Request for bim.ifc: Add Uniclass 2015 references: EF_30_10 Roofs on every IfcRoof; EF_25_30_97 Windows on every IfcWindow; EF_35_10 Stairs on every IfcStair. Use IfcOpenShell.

First a look at what the model holds.

```python
import ifcopenshell

model = ifcopenshell.open("bim.ifc")
print(model.schema)
print("classifications:", [c.Name for c in model.by_type("IfcClassification")])
for ifc_class in ("IfcDoor", "IfcRoof", "IfcStair", "IfcWall", "IfcWindow"):
    print(ifc_class, len(model.by_type(ifc_class)))
```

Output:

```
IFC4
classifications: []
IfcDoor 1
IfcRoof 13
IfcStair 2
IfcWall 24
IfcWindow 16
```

```python
import ifcopenshell
import ifcopenshell.api.classification

model = ifcopenshell.open("bim.ifc")

system = ifcopenshell.api.classification.add_classification(model, classification="Uniclass 2015")

codes = {
    "IfcRoof": ("EF_30_10", "Roofs"),
    "IfcWindow": ("EF_25_30_97", "Windows"),
    "IfcStair": ("EF_35_10", "Stairs"),
}
for ifc_class, (code, name) in codes.items():
    products = model.by_type(ifc_class)
    ifcopenshell.api.classification.add_reference(
        model, products=products, classification=system, identification=code, name=name
    )
    print(code, len(products))

model.write("bim-out.ifc")
```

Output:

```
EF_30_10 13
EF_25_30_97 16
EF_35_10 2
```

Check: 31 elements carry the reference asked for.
